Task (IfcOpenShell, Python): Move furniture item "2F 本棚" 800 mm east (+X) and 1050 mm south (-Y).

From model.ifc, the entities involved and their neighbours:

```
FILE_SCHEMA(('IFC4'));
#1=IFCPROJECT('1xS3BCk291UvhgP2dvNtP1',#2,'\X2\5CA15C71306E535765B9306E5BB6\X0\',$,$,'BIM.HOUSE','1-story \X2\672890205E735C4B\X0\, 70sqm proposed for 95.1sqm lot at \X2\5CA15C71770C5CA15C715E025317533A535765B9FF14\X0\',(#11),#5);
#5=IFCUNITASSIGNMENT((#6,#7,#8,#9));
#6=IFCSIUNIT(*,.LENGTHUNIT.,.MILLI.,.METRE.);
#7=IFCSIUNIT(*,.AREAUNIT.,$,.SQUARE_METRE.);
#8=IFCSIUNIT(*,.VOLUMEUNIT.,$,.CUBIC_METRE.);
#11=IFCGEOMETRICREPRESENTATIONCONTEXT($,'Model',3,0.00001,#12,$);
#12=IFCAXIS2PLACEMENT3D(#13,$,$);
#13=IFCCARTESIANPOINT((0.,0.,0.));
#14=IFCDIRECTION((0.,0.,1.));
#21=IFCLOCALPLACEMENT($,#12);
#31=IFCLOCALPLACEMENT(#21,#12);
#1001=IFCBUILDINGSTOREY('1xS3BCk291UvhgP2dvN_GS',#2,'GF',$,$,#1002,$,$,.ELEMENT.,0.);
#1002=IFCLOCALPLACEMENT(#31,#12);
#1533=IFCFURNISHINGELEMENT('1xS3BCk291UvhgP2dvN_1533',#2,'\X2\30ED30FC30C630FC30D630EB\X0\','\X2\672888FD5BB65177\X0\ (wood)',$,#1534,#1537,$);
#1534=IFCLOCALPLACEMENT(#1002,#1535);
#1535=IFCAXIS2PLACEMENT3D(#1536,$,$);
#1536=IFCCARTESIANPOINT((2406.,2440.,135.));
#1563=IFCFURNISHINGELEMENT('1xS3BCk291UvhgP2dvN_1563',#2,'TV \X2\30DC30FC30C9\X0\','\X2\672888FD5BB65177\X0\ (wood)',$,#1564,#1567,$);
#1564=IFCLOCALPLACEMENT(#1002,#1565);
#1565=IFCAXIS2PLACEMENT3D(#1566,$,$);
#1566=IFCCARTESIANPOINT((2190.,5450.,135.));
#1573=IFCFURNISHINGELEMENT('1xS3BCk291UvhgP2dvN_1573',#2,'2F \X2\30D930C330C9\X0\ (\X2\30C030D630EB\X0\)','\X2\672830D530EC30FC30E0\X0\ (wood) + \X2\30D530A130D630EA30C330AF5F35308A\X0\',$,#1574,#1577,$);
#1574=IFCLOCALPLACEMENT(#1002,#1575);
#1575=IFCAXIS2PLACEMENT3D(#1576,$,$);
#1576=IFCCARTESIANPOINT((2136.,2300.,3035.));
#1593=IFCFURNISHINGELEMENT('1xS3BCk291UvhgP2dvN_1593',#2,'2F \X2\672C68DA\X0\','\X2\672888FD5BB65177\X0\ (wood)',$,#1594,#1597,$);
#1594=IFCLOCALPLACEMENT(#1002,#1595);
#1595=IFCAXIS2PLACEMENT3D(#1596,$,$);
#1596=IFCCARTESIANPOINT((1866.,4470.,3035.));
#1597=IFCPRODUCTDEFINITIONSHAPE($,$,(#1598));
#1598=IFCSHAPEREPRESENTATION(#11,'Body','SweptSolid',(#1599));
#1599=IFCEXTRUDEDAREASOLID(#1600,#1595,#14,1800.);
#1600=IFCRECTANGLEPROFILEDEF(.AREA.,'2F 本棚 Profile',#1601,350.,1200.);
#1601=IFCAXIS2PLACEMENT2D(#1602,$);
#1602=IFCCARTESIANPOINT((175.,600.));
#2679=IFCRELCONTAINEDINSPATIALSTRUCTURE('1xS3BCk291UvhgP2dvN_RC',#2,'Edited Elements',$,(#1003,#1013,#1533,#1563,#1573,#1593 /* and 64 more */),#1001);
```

```python
import ifcopenshell
import ifcopenshell.api.geometry
import ifcopenshell.util.placement

model = ifcopenshell.open("model.ifc")

item = model.by_guid("1xS3BCk291UvhgP2dvN_1593")
matrix = ifcopenshell.util.placement.get_local_placement(item.ObjectPlacement)
matrix[0, 3] += 800.0
matrix[1, 3] -= 1050.0
ifcopenshell.api.geometry.edit_object_placement(model, product=item, matrix=matrix, is_si=False)

print(ifcopenshell.util.placement.get_local_placement(item.ObjectPlacement).round(3) + 0.0)

model.write("model_edited.ifc")
```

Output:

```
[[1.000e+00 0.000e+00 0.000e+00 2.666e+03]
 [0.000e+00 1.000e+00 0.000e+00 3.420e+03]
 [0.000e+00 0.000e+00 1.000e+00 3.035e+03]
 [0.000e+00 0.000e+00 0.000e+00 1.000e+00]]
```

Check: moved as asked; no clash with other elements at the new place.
